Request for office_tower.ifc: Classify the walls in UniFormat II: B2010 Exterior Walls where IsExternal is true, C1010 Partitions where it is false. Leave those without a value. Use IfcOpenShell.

First a look at what the model holds.

```python
import ifcopenshell
import ifcopenshell.util.element

model = ifcopenshell.open("office_tower.ifc")
print(model.schema)
print("classifications:", [c.Name for c in model.by_type("IfcClassification")])
values = [ifcopenshell.util.element.get_pset(e, "Pset_WallCommon", "IsExternal") for e in model.by_type("IfcWall")]
for value in (True, False, None):
    print("IsExternal", value, values.count(value))
```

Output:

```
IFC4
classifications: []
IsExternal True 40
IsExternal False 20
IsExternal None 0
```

```python
import ifcopenshell
import ifcopenshell.api.classification
import ifcopenshell.util.element

model = ifcopenshell.open("office_tower.ifc")

system = ifcopenshell.api.classification.add_classification(model, classification="UniFormat II")

walls = model.by_type("IfcWall")
external = {e: ifcopenshell.util.element.get_pset(e, "Pset_WallCommon", "IsExternal") for e in walls}
for flag, code, name in ((True, "B2010", "Exterior Walls"), (False, "C1010", "Partitions")):
    products = [e for e in walls if external[e] is flag]
    ifcopenshell.api.classification.add_reference(
        model, products=products, classification=system, identification=code, name=name
    )
    print(code, len(products))

model.write("office_tower_rev.ifc")
```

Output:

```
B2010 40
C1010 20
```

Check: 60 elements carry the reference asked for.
